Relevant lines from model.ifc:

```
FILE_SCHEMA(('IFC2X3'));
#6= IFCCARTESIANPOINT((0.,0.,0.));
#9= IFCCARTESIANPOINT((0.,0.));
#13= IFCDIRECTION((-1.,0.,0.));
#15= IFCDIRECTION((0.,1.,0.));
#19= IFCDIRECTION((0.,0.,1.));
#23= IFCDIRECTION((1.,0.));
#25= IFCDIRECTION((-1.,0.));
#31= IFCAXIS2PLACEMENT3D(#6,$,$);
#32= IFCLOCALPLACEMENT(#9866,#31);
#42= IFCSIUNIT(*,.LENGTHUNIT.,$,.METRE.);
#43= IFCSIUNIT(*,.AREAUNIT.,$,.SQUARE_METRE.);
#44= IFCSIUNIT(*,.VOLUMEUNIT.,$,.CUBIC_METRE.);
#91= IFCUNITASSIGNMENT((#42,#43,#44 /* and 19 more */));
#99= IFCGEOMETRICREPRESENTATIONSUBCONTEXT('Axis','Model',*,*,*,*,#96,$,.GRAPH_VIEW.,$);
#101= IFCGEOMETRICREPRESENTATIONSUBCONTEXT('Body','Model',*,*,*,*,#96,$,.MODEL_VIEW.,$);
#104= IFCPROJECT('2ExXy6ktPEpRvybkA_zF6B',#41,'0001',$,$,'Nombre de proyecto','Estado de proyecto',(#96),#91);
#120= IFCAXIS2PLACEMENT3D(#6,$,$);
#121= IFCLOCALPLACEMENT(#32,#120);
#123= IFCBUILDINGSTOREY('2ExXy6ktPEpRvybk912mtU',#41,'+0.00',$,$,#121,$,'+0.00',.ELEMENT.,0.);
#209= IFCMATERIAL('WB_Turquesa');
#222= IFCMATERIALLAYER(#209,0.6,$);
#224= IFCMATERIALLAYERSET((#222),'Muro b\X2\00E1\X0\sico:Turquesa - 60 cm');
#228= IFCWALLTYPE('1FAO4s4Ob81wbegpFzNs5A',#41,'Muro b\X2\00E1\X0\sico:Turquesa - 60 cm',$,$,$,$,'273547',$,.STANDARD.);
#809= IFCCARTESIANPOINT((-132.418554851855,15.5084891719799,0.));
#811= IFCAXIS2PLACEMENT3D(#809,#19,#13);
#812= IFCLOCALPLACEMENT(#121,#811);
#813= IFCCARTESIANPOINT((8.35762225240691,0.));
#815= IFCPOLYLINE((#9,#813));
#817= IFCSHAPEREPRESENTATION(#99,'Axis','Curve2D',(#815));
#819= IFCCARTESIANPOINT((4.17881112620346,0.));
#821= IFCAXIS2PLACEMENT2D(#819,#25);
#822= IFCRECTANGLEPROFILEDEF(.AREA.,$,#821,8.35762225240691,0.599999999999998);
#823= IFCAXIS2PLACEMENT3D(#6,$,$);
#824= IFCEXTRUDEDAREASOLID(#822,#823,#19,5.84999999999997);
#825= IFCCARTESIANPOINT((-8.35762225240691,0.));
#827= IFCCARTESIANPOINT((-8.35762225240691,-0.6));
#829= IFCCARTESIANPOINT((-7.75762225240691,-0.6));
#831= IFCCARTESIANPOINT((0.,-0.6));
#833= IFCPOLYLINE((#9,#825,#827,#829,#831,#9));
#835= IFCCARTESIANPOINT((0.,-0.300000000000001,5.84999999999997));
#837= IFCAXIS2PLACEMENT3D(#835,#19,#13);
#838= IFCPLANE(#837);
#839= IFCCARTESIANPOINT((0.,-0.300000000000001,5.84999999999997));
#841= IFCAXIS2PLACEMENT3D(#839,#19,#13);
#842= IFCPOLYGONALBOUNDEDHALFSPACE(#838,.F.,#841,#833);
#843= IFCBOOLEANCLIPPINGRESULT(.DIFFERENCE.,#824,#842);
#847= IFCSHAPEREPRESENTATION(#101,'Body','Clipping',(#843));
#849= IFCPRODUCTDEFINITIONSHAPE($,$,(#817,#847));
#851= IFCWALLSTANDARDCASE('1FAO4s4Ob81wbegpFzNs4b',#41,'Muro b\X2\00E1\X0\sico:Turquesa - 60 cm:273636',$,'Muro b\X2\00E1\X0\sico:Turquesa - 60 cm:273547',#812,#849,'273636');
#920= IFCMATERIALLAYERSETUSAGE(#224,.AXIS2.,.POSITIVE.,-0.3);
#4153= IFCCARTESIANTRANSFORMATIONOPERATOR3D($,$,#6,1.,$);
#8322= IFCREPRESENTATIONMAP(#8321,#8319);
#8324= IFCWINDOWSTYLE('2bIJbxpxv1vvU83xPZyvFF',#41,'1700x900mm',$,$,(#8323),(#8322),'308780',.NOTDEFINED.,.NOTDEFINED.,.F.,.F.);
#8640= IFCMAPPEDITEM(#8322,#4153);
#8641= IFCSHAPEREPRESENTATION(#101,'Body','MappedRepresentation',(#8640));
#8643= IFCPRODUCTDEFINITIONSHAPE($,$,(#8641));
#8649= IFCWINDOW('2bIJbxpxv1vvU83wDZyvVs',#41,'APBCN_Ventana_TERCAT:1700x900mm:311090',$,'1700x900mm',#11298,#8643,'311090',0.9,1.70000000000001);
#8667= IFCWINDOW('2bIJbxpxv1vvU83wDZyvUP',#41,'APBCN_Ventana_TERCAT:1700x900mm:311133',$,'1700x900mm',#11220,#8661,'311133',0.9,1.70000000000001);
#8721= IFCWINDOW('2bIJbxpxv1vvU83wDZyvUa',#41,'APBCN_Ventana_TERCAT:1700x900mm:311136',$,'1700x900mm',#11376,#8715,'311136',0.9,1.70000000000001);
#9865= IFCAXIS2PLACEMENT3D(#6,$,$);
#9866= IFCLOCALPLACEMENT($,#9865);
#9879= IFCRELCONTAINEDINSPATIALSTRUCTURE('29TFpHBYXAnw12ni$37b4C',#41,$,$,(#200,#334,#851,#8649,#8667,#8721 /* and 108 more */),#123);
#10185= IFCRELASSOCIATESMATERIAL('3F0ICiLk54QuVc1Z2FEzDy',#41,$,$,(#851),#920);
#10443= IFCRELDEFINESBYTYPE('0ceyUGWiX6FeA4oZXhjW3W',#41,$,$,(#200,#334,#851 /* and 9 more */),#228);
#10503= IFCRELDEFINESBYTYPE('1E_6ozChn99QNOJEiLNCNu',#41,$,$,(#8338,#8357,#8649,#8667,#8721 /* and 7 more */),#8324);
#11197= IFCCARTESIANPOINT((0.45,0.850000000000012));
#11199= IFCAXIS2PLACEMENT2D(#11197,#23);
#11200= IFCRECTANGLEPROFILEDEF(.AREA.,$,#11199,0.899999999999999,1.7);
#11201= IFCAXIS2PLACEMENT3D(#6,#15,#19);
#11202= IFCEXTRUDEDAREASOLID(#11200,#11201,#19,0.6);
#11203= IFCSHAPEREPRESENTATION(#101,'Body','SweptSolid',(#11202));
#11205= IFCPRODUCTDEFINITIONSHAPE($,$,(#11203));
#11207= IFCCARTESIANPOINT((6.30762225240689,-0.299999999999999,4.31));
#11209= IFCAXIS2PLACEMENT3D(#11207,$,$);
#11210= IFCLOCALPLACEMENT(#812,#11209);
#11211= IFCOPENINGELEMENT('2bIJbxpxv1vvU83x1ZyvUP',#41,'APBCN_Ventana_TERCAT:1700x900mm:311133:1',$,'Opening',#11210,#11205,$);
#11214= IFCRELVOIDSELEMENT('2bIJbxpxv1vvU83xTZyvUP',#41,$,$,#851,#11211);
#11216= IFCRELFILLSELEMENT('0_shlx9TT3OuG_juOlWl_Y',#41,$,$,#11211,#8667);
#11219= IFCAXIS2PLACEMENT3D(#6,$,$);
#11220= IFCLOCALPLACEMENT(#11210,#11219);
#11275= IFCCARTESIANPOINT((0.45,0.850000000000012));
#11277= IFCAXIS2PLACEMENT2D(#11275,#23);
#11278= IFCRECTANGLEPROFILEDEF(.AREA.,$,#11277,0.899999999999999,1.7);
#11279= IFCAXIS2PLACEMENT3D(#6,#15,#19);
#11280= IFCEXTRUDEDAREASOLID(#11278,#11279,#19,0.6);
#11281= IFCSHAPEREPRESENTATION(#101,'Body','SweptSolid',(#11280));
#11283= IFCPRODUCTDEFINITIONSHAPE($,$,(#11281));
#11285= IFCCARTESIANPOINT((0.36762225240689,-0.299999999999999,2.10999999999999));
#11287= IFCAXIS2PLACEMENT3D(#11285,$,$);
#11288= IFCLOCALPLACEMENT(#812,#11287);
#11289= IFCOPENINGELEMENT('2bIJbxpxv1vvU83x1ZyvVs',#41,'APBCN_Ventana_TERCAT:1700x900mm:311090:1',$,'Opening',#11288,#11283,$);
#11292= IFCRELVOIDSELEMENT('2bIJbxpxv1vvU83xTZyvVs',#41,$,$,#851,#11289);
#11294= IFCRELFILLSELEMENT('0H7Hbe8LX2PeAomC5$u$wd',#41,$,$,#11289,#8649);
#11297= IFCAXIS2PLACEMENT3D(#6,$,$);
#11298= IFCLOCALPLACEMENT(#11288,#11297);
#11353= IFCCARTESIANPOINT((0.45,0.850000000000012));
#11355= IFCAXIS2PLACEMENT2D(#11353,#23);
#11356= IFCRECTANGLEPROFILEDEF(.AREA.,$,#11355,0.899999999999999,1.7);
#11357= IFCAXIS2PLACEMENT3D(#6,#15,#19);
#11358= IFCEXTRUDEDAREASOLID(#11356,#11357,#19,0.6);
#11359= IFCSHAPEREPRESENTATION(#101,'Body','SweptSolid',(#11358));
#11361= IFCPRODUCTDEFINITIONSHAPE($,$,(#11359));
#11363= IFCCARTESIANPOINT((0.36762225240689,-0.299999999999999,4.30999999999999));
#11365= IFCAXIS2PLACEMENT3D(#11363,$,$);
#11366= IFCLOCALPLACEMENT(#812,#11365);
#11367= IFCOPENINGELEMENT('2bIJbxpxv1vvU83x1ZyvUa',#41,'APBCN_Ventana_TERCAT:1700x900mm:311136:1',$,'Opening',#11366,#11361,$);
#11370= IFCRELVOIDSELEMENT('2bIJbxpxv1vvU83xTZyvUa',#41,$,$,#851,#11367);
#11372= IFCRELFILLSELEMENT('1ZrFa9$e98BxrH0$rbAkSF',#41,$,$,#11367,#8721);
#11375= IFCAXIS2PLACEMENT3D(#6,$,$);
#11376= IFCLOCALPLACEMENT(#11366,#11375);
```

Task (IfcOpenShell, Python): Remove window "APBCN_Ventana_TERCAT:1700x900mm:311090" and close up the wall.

```python
import ifcopenshell
import ifcopenshell.api.feature
import ifcopenshell.api.root
import ifcopenshell.geom
import ifcopenshell.util.shape

model = ifcopenshell.open("model.ifc")
settings = ifcopenshell.geom.settings()


def volume(element):
    """Net volume in cubic metres, openings subtracted."""
    shape = ifcopenshell.geom.create_shape(settings, element)
    return ifcopenshell.util.shape.get_volume(shape.geometry)


window = model.by_guid("2bIJbxpxv1vvU83wDZyvVs")
opening = window.FillsVoids[0].RelatingOpeningElement
wall = opening.VoidsElements[0].RelatingBuildingElement
before = volume(wall)

ifcopenshell.api.root.remove_product(model, product=window)
ifcopenshell.api.feature.remove_feature(model, feature=opening)

after = volume(wall)

print(f"wall volume {before:.3f} -> {after:.3f} m3")

model.write("model_updated.ifc")
```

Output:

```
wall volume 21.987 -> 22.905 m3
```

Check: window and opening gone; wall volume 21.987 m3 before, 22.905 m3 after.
